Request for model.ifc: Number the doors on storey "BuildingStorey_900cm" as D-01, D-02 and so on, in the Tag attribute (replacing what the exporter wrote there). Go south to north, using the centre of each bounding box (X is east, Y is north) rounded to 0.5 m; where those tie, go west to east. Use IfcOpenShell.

First a look at what the model holds.

```python
import ifcopenshell
import ifcopenshell.util.element
import ifcopenshell.util.placement

model = ifcopenshell.open("model.ifc")
print(model.schema)
storey = next(s for s in model.by_type("IfcBuildingStorey") if s.Name == "BuildingStorey_900cm")
doors = [e for e in ifcopenshell.util.element.get_decomposition(storey) if e.is_a("IfcDoor")]
for e in sorted(doors, key=lambda e: e.id()):
    origin = ifcopenshell.util.placement.get_local_placement(e.ObjectPlacement)[:3, 3]
    print(e.id(), e.Tag, e.Name, origin.round(2) + 0.0, sep=" | ")
```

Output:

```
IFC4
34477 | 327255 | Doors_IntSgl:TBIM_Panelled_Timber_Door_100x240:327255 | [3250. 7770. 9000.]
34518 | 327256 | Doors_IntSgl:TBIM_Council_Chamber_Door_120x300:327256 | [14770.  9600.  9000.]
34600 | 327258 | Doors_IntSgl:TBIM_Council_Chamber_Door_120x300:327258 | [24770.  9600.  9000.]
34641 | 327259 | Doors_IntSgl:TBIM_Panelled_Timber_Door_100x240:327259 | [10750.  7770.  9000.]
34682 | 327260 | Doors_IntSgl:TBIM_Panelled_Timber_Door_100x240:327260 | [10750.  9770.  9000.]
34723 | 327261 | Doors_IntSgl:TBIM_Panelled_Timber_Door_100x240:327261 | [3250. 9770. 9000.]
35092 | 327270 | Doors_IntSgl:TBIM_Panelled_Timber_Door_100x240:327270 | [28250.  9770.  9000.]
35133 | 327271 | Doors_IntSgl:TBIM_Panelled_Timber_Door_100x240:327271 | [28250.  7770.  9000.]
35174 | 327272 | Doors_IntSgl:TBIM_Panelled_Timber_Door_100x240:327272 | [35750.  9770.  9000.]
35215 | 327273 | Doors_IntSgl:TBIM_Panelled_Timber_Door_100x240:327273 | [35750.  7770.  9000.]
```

```python
import ifcopenshell
import ifcopenshell.geom
import ifcopenshell.util.element
import ifcopenshell.util.shape

model = ifcopenshell.open("model.ifc")
settings = ifcopenshell.geom.settings()
settings.set("use-world-coords", True)


def centre(element):
    shape = ifcopenshell.geom.create_shape(settings, element)
    return ifcopenshell.util.shape.get_bbox_centroid(shape.geometry)


storey = next(s for s in model.by_type("IfcBuildingStorey") if s.Name == "BuildingStorey_900cm")
doors = [e for e in ifcopenshell.util.element.get_decomposition(storey) if e.is_a("IfcDoor")]

# Insertion points can sit at a corner or the storey origin, so sort by the geometry (in metres).
centres = {e: centre(e) for e in doors}
doors.sort(key=lambda e: (round(centres[e][1] / 0.5), centres[e][0]))

for i, e in enumerate(doors, start=1):
    number = f"D-{i:02d}"
    e.Tag = number
    print(e.id(), number)

model.write("model_v2.ifc")
```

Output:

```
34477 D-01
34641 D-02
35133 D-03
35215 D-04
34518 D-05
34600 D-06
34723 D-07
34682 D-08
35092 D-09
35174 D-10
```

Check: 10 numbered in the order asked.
